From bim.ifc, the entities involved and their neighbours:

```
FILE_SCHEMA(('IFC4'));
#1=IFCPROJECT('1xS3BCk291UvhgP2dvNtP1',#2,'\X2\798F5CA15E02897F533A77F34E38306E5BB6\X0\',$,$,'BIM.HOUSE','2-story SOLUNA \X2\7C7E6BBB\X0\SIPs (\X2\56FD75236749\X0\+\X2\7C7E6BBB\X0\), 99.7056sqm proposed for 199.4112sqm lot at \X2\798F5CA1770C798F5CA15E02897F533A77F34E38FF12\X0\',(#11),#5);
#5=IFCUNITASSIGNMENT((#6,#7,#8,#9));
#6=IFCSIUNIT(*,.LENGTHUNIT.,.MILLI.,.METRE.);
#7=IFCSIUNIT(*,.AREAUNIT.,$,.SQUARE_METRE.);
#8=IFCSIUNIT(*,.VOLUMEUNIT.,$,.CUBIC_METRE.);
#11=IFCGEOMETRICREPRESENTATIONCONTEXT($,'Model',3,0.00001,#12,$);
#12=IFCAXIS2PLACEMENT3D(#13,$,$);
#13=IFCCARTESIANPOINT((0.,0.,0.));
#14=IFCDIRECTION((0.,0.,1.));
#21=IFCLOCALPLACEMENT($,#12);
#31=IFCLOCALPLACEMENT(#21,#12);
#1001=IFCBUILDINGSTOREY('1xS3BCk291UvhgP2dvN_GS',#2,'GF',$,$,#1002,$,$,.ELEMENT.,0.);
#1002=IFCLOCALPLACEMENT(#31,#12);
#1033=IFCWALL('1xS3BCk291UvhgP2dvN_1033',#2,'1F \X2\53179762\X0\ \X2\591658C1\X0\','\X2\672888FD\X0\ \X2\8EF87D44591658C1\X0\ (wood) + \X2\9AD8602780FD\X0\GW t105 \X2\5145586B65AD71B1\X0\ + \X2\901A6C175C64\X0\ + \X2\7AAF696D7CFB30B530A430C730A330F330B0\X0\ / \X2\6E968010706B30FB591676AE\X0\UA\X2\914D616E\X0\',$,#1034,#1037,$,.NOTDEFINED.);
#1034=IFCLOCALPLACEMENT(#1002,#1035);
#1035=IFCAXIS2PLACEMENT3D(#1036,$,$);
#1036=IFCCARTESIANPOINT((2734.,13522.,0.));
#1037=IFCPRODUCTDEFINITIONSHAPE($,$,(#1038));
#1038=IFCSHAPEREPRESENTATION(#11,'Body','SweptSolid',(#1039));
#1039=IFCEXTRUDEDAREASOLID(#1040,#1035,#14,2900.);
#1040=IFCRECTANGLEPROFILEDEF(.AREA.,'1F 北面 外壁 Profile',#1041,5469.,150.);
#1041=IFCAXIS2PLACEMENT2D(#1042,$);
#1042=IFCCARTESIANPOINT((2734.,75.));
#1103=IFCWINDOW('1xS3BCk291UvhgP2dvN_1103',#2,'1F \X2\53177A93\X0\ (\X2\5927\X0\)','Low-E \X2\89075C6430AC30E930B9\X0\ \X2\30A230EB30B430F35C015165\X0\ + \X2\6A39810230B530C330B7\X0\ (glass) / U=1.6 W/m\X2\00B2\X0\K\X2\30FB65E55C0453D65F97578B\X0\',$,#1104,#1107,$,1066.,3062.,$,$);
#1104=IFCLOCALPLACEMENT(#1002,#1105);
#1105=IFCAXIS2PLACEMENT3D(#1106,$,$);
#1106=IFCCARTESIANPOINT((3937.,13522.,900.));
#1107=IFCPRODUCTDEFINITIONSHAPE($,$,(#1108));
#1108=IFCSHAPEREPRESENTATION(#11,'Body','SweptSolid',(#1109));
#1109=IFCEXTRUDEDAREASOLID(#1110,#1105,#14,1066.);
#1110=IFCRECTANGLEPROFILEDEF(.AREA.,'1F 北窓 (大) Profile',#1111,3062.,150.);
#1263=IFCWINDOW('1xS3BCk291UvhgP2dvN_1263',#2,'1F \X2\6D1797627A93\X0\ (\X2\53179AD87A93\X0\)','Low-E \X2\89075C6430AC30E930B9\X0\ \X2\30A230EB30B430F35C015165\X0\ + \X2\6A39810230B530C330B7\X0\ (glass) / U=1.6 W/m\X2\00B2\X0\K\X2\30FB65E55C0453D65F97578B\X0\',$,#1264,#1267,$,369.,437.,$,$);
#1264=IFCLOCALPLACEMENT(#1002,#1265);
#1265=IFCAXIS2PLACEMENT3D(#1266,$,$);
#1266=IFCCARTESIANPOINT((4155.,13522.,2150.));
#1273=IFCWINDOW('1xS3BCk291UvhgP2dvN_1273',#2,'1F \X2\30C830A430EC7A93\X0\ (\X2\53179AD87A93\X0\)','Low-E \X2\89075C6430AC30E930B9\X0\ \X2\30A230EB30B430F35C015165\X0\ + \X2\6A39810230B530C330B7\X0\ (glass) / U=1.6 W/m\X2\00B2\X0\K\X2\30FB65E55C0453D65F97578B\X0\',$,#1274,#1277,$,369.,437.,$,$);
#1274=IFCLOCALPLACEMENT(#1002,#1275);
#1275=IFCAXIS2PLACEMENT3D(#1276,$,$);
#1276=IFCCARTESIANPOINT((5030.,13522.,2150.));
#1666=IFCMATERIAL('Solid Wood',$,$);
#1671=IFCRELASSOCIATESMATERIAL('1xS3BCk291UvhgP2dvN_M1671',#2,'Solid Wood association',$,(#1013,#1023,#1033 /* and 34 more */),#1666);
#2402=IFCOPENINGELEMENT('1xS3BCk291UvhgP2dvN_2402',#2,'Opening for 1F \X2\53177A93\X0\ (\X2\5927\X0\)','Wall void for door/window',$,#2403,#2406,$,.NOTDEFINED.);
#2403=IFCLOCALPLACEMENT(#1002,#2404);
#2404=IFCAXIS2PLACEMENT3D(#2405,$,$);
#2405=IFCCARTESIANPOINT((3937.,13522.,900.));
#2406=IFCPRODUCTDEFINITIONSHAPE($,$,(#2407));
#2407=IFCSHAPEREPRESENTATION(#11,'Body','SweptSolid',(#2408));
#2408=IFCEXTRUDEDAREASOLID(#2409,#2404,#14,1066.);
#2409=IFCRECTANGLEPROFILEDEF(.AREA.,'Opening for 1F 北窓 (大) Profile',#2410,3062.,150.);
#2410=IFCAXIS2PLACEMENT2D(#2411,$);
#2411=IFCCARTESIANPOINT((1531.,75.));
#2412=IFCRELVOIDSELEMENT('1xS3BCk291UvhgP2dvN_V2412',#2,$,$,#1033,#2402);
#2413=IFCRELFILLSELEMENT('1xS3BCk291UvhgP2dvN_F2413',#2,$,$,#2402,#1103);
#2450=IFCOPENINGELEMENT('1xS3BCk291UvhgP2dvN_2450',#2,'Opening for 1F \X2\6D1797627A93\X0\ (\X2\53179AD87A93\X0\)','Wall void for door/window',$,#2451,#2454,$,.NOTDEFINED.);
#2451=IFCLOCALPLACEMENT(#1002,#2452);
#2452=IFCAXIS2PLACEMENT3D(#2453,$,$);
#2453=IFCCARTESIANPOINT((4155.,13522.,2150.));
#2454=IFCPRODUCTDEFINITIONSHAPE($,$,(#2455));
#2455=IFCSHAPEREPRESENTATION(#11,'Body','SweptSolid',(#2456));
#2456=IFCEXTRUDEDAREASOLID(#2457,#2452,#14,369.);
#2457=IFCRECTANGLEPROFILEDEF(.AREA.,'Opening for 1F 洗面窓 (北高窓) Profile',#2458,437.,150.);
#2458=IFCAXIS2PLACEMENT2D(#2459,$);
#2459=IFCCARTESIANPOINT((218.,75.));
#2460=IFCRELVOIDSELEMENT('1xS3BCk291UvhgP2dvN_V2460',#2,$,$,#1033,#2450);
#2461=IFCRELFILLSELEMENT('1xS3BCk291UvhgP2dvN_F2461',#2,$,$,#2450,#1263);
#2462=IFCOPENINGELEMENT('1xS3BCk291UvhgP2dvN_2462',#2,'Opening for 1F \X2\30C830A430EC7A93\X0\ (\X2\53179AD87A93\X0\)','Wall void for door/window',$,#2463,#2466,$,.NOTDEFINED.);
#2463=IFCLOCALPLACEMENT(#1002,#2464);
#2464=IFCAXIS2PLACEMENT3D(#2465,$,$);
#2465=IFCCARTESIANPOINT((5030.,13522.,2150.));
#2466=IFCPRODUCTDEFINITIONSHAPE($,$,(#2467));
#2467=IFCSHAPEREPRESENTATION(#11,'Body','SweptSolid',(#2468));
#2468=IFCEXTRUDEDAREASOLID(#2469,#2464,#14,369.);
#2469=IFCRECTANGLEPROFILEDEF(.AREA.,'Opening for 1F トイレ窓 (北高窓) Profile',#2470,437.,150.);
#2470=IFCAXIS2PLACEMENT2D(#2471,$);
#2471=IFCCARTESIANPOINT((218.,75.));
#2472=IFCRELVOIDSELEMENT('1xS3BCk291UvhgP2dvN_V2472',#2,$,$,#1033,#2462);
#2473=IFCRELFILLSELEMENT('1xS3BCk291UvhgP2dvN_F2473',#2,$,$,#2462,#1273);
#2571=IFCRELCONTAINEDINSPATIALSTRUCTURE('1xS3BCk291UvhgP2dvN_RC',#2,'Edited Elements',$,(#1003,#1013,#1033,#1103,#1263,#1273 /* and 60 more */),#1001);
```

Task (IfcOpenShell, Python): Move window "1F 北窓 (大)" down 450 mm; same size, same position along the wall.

```python
import numpy as np
import ifcopenshell
import ifcopenshell.api.geometry
import ifcopenshell.util.placement
import ifcopenshell.util.unit

model = ifcopenshell.open("bim.ifc")
unit_scale = ifcopenshell.util.unit.calculate_unit_scale(model)

window = model.by_guid("1xS3BCk291UvhgP2dvN_1103")
opening = window.FillsVoids[0].RelatingOpeningElement
dz = -0.45 / unit_scale

shift = np.array([0.0, 0.0, dz])
# The window is not placed relative to its opening, so move both.
for product in (opening, window):
    matrix = ifcopenshell.util.placement.get_local_placement(product.ObjectPlacement)
    matrix[:3, 3] += shift
    ifcopenshell.api.geometry.edit_object_placement(model, product=product, matrix=matrix, is_si=False)

print(f"moved by {dz * unit_scale:+.3f} m")

model.write("bim_updated.ifc")
```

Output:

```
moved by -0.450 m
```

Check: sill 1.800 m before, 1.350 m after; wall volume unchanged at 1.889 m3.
